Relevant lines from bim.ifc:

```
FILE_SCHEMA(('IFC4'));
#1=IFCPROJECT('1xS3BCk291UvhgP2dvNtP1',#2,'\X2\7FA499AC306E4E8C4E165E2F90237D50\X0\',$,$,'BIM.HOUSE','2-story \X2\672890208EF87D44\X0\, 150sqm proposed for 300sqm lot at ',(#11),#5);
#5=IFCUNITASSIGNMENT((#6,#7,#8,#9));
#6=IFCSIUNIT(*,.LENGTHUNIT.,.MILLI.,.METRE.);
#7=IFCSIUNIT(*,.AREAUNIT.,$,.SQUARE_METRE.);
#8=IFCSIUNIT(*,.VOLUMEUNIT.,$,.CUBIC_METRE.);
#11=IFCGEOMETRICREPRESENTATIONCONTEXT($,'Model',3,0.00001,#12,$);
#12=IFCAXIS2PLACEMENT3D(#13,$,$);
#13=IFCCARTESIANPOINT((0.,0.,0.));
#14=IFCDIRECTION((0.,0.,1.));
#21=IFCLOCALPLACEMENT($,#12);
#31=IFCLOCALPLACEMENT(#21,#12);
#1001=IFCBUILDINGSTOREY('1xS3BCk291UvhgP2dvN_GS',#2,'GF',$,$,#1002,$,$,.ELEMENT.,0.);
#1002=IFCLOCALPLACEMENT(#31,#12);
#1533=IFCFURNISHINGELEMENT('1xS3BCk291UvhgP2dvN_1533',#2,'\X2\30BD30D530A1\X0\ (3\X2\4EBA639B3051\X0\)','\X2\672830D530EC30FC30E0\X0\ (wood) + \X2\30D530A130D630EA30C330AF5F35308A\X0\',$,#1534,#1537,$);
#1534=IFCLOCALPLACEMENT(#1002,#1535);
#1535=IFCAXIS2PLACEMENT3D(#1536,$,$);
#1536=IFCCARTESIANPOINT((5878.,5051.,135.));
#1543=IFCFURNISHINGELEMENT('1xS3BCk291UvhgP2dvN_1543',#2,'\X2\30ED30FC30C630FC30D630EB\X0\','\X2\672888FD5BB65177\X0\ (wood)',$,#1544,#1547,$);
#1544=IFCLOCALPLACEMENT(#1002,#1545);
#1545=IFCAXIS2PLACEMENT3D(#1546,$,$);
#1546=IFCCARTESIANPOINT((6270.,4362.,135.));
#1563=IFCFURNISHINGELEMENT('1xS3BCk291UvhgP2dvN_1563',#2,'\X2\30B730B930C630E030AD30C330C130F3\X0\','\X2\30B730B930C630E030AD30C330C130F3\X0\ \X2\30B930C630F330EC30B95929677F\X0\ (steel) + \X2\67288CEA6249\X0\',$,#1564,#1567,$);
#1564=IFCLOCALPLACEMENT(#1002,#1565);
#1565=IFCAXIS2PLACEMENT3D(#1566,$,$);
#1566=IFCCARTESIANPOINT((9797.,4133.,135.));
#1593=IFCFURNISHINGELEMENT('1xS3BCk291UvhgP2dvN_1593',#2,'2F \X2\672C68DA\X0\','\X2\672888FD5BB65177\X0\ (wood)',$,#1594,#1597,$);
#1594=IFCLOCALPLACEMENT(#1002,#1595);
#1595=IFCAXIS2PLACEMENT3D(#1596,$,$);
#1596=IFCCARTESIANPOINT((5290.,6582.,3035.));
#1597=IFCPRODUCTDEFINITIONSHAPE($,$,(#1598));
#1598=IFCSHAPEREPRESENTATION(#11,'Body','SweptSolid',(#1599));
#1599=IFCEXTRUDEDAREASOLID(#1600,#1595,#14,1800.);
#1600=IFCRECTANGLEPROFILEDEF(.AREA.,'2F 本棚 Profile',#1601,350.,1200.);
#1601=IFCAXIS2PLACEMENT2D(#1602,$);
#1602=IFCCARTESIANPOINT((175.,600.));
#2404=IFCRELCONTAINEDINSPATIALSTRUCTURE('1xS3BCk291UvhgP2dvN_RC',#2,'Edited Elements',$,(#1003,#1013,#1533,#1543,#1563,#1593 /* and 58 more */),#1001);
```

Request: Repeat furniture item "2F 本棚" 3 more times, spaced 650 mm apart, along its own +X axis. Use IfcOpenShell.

```python
import ifcopenshell
import ifcopenshell.api.geometry
import ifcopenshell.api.root
import ifcopenshell.util.element
import ifcopenshell.util.placement
import ifcopenshell.util.unit

model = ifcopenshell.open("bim.ifc")
unit_scale = ifcopenshell.util.unit.calculate_unit_scale(model)


def reuse_history(source, copy):
    """copy_class also copies each property set's owner history, people and application; keep the originals."""
    for rel in copy.IsDefinedBy:
        if rel.is_a("IfcRelDefinesByProperties") and (history := rel.RelatingPropertyDefinition.OwnerHistory):
            rel.RelatingPropertyDefinition.OwnerHistory = source.OwnerHistory
            ifcopenshell.util.element.remove_deep2(model, history)


source = model.by_id(1593)
base = ifcopenshell.util.placement.get_local_placement(source.ObjectPlacement)
step = base[:3, 0] * 0.65 / unit_scale

for i in range(1, 4):
    copy = ifcopenshell.api.root.copy_class(model, product=source)
    copy.Representation = ifcopenshell.util.element.copy_deep(
        model, source.Representation, exclude=["IfcGeometricRepresentationContext", "IfcRepresentationMap"]
    )
    reuse_history(source, copy)
    matrix = base.copy()
    matrix[:3, 3] += i * step
    print("added at", matrix[:3, 3].round(3) + 0.0)
    ifcopenshell.api.geometry.edit_object_placement(model, product=copy, matrix=matrix, is_si=False)

model.write("bim_rev.ifc")
```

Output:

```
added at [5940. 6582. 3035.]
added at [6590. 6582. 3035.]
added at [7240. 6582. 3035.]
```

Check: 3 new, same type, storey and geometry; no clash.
